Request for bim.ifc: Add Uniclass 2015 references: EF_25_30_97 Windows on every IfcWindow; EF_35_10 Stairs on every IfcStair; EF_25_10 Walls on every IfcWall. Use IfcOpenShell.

First a look at what the model holds.

```python
import ifcopenshell

model = ifcopenshell.open("bim.ifc")
print(model.schema)
print("classifications:", [c.Name for c in model.by_type("IfcClassification")])
for ifc_class in ("IfcDoor", "IfcRoof", "IfcStair", "IfcWall", "IfcWindow"):
    print(ifc_class, len(model.by_type(ifc_class)))
```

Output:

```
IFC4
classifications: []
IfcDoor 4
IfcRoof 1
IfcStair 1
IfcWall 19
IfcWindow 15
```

```python
import ifcopenshell
import ifcopenshell.api.classification

model = ifcopenshell.open("bim.ifc")

system = ifcopenshell.api.classification.add_classification(model, classification="Uniclass 2015")

codes = {
    "IfcWindow": ("EF_25_30_97", "Windows"),
    "IfcStair": ("EF_35_10", "Stairs"),
    "IfcWall": ("EF_25_10", "Walls"),
}
for ifc_class, (code, name) in codes.items():
    products = model.by_type(ifc_class)
    ifcopenshell.api.classification.add_reference(
        model, products=products, classification=system, identification=code, name=name
    )
    print(code, len(products))

model.write("bim_edited.ifc")
```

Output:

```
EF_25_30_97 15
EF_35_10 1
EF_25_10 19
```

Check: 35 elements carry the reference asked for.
